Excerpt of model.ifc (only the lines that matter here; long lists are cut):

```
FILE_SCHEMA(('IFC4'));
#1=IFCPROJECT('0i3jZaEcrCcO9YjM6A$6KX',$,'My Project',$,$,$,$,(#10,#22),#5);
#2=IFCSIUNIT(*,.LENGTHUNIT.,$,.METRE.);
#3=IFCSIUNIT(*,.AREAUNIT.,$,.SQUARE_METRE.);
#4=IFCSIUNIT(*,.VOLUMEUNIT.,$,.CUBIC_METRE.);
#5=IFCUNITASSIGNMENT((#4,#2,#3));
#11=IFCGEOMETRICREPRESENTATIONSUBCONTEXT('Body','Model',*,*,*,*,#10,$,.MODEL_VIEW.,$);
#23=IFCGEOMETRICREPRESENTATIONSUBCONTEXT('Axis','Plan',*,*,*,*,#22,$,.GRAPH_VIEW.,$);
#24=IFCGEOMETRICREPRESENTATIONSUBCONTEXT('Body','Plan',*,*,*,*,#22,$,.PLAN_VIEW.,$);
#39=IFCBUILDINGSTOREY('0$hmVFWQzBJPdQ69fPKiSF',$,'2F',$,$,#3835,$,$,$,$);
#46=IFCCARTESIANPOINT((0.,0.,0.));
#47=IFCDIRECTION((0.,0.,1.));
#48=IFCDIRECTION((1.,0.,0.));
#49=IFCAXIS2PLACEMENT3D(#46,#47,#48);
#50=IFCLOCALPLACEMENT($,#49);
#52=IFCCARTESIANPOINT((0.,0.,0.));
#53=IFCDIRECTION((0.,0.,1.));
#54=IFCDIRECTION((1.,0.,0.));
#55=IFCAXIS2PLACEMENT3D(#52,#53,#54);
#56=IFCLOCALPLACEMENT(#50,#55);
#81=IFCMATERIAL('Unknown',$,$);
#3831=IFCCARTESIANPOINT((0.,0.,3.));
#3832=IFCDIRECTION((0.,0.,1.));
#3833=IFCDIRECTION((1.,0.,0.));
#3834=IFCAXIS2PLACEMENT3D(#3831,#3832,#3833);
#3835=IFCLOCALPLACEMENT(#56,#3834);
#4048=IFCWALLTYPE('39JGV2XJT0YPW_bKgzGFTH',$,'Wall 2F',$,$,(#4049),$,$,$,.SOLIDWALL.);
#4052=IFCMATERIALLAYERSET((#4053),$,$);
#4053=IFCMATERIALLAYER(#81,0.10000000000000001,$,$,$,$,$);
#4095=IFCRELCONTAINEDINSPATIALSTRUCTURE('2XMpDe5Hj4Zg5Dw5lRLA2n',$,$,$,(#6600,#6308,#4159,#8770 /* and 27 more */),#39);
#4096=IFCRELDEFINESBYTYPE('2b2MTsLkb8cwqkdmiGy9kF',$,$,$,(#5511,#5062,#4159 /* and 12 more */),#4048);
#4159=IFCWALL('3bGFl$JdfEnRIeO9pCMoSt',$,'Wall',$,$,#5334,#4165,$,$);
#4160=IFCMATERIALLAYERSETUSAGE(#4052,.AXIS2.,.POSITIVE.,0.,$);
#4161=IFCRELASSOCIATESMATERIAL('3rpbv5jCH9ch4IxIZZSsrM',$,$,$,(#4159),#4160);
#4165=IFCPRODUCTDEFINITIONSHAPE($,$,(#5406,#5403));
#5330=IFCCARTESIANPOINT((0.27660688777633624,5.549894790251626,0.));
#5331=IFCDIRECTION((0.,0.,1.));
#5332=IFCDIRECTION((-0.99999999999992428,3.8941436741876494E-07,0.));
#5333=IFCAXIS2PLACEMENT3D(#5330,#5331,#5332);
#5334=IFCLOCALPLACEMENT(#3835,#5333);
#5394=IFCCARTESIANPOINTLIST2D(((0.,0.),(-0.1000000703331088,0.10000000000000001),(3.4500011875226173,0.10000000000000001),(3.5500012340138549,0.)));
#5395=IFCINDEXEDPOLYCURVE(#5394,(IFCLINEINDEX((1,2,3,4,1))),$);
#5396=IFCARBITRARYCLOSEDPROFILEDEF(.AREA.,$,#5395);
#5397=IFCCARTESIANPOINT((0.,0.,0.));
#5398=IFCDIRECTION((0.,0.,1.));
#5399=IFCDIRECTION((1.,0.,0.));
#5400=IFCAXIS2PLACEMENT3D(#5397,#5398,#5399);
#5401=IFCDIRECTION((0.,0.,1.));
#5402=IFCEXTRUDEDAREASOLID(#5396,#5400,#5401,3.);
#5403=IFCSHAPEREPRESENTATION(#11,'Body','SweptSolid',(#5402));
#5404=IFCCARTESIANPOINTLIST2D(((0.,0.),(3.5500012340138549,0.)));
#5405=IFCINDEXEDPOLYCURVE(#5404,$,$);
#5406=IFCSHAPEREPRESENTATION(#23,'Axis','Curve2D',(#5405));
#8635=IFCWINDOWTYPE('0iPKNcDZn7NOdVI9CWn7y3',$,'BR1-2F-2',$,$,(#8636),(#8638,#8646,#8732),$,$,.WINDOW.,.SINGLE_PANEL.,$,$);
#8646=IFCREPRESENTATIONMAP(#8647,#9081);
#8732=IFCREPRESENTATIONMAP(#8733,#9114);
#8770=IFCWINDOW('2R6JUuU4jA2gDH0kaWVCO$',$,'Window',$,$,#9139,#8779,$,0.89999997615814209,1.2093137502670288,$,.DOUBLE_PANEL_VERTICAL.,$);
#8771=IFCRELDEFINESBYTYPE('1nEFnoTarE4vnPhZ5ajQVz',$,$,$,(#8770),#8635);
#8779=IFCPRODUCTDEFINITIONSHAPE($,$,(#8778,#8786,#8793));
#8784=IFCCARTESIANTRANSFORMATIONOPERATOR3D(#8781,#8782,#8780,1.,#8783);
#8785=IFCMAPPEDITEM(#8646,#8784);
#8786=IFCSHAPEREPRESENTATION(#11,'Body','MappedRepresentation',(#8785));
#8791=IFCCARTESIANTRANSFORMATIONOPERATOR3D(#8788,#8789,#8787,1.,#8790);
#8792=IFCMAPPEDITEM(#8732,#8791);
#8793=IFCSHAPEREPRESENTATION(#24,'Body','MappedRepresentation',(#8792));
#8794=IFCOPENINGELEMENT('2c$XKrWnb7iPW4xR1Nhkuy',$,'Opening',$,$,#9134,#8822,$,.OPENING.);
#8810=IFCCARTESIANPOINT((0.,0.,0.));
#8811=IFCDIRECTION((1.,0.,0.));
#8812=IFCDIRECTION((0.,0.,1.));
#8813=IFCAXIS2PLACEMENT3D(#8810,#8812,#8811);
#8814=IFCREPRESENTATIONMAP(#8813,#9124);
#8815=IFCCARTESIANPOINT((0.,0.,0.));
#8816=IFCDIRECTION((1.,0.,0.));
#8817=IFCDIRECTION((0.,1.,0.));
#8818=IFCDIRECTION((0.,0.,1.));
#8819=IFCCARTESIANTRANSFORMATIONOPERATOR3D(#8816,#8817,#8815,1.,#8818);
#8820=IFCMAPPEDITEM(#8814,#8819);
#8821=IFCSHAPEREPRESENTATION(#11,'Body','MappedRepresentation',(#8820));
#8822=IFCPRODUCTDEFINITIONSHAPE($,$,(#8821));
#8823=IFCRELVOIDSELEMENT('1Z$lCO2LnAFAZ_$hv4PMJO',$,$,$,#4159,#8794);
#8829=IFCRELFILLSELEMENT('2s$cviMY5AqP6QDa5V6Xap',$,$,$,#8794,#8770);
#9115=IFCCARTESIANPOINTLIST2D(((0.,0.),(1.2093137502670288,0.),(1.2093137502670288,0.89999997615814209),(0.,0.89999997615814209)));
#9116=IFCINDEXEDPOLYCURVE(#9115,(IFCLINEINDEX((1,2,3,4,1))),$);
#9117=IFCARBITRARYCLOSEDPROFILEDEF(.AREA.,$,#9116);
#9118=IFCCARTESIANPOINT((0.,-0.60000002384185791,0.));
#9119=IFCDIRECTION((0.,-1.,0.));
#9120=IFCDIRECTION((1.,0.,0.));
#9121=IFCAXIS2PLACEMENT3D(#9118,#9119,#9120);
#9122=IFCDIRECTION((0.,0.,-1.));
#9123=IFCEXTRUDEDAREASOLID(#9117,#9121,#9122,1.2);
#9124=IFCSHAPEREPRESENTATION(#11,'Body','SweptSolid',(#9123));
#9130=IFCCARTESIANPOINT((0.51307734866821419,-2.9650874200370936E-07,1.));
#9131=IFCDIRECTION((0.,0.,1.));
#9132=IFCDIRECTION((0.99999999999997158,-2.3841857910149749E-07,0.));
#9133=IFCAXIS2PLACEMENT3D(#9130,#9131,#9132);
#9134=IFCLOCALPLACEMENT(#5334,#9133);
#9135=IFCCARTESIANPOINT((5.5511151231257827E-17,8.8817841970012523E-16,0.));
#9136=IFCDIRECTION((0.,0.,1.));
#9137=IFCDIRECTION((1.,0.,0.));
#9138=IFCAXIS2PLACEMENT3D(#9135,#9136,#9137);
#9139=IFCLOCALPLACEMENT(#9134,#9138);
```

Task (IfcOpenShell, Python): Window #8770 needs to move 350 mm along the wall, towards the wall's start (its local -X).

```python
import ifcopenshell
import ifcopenshell.api.geometry
import ifcopenshell.util.placement
import ifcopenshell.util.unit

model = ifcopenshell.open("model.ifc")
unit_scale = ifcopenshell.util.unit.calculate_unit_scale(model)

window = model.by_id(8770)
opening = window.FillsVoids[0].RelatingOpeningElement
wall = opening.VoidsElements[0].RelatingBuildingElement

wall_matrix = ifcopenshell.util.placement.get_local_placement(wall.ObjectPlacement)
shift = wall_matrix[:3, 0] * -0.35 / unit_scale
before = ifcopenshell.util.placement.get_local_placement(window.ObjectPlacement)[:3, 3].copy()

# The window is placed relative to its opening, so it follows when the opening moves.
matrix = ifcopenshell.util.placement.get_local_placement(opening.ObjectPlacement)
matrix[:3, 3] += shift
ifcopenshell.api.geometry.edit_object_placement(
    model, product=opening, matrix=matrix, is_si=False, should_transform_children=True
)

after = ifcopenshell.util.placement.get_local_placement(window.ObjectPlacement)[:3, 3]
print("window moved by", (after - before).round(3) + 0.0)

model.write("model_rev.ifc")
```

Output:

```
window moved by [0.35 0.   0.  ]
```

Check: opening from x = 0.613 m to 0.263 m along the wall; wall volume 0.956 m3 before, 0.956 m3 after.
